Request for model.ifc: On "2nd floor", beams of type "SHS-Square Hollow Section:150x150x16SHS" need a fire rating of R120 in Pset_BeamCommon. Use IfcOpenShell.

First a look at what the model holds.

```python
import ifcopenshell
import ifcopenshell.util.element

model = ifcopenshell.open("model.ifc")
print(model.schema)
storey = next(s for s in model.by_type("IfcBuildingStorey") if s.Name == "2nd floor")
beams = [e for e in ifcopenshell.util.element.get_decomposition(storey) if e.is_a("IfcBeam")]
seen = {}
for e in beams:
    element_type = ifcopenshell.util.element.get_type(e)
    key = (element_type.Name if element_type != e and element_type else None, ifcopenshell.util.element.get_pset(e, "Pset_BeamCommon", "FireRating"))
    seen[key] = seen.get(key, 0) + 1
for (name, value), count in sorted(seen.items(), key=str):
    print(count, "x", name, "|", value)
```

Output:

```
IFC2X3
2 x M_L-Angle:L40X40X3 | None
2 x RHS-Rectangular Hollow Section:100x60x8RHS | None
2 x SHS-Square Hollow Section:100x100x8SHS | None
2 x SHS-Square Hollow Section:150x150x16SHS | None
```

```python
import ifcopenshell
import ifcopenshell.api.pset
import ifcopenshell.util.element

model = ifcopenshell.open("model.ifc")

storey = next(s for s in model.by_type("IfcBuildingStorey") if s.Name == "2nd floor")
beams = [e for e in ifcopenshell.util.element.get_decomposition(storey) if e.is_a("IfcBeam")]

count = 0
for e in beams:
    element_type = ifcopenshell.util.element.get_type(e)
    if element_type in (None, e) or element_type.Name != "SHS-Square Hollow Section:150x150x16SHS":
        continue
    # add_pset returns the element's existing set when there is one.
    pset = ifcopenshell.api.pset.add_pset(model, product=e, name="Pset_BeamCommon")
    ifcopenshell.api.pset.edit_pset(model, pset=pset, properties={"FireRating": "R120"})
    count += 1

print(count, "beams updated")

model.write("model_v2.ifc")
```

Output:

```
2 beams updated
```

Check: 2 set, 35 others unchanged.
